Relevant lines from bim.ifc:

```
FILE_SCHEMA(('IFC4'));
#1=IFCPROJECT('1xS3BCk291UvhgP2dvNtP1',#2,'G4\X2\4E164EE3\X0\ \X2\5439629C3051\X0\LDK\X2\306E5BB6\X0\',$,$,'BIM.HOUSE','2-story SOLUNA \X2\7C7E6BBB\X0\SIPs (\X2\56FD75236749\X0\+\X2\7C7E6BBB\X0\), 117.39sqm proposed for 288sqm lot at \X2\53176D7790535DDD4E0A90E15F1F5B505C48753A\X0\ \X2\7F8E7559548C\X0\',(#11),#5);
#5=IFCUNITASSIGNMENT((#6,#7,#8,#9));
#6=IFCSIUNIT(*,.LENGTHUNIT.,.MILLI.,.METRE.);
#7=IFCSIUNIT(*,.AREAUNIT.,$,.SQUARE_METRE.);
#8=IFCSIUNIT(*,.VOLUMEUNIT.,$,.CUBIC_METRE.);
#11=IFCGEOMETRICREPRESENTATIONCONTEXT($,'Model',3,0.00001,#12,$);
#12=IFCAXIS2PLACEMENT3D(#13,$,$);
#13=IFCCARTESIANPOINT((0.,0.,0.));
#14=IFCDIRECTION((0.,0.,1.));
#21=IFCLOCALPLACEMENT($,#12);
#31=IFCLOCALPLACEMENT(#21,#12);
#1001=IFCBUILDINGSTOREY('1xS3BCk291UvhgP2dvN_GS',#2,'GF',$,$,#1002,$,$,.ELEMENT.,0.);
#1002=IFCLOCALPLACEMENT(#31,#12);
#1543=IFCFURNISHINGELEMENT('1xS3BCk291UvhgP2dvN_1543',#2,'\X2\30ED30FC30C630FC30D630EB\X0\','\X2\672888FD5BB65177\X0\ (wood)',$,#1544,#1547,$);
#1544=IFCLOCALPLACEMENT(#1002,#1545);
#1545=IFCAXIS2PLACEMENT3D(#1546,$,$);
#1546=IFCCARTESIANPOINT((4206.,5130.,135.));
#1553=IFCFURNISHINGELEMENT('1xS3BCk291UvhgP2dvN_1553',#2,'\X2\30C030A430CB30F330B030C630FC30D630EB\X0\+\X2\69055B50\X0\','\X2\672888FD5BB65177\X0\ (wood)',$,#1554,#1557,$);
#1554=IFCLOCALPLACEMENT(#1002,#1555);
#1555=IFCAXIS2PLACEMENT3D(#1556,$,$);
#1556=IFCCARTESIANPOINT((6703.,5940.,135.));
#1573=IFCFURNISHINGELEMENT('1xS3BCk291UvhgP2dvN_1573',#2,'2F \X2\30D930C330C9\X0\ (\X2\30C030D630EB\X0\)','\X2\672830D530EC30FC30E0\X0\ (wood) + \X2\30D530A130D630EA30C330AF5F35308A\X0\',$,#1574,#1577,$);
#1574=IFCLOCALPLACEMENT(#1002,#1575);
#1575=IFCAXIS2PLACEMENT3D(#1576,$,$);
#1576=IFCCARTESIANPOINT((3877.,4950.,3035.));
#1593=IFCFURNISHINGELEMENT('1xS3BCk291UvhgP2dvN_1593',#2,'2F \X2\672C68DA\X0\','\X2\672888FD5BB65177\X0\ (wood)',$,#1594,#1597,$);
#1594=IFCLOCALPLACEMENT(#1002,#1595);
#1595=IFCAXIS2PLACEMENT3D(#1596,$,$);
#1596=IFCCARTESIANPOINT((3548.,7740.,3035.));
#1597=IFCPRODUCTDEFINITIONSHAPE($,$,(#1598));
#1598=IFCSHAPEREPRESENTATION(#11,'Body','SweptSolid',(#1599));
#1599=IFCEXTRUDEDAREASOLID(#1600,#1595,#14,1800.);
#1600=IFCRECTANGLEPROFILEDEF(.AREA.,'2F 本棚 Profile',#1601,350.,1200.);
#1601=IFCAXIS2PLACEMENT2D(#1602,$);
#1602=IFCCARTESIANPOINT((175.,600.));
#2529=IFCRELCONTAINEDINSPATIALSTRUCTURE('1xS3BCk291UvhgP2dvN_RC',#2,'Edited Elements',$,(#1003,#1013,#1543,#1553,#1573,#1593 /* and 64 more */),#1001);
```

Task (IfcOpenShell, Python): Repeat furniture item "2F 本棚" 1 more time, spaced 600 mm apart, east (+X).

```python
import numpy as np
import ifcopenshell
import ifcopenshell.api.geometry
import ifcopenshell.api.root
import ifcopenshell.util.element
import ifcopenshell.util.placement

model = ifcopenshell.open("bim.ifc")


def reuse_history(source, copy):
    """copy_class also copies each property set's owner history, people and application; keep the originals."""
    for rel in copy.IsDefinedBy:
        if rel.is_a("IfcRelDefinesByProperties") and (history := rel.RelatingPropertyDefinition.OwnerHistory):
            rel.RelatingPropertyDefinition.OwnerHistory = source.OwnerHistory
            ifcopenshell.util.element.remove_deep2(model, history)


source = model.by_guid("1xS3BCk291UvhgP2dvN_1593")
base = ifcopenshell.util.placement.get_local_placement(source.ObjectPlacement)
step = np.array([1.0, 0.0, 0.0]) * 600.0

for i in range(1, 2):
    copy = ifcopenshell.api.root.copy_class(model, product=source)
    copy.Representation = ifcopenshell.util.element.copy_deep(
        model, source.Representation, exclude=["IfcGeometricRepresentationContext", "IfcRepresentationMap"]
    )
    reuse_history(source, copy)
    matrix = base.copy()
    matrix[:3, 3] += i * step
    print("added at", matrix[:3, 3].round(3) + 0.0)
    ifcopenshell.api.geometry.edit_object_placement(model, product=copy, matrix=matrix, is_si=False)

model.write("bim_v2.ifc")
```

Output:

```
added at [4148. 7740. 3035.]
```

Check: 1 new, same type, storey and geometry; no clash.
